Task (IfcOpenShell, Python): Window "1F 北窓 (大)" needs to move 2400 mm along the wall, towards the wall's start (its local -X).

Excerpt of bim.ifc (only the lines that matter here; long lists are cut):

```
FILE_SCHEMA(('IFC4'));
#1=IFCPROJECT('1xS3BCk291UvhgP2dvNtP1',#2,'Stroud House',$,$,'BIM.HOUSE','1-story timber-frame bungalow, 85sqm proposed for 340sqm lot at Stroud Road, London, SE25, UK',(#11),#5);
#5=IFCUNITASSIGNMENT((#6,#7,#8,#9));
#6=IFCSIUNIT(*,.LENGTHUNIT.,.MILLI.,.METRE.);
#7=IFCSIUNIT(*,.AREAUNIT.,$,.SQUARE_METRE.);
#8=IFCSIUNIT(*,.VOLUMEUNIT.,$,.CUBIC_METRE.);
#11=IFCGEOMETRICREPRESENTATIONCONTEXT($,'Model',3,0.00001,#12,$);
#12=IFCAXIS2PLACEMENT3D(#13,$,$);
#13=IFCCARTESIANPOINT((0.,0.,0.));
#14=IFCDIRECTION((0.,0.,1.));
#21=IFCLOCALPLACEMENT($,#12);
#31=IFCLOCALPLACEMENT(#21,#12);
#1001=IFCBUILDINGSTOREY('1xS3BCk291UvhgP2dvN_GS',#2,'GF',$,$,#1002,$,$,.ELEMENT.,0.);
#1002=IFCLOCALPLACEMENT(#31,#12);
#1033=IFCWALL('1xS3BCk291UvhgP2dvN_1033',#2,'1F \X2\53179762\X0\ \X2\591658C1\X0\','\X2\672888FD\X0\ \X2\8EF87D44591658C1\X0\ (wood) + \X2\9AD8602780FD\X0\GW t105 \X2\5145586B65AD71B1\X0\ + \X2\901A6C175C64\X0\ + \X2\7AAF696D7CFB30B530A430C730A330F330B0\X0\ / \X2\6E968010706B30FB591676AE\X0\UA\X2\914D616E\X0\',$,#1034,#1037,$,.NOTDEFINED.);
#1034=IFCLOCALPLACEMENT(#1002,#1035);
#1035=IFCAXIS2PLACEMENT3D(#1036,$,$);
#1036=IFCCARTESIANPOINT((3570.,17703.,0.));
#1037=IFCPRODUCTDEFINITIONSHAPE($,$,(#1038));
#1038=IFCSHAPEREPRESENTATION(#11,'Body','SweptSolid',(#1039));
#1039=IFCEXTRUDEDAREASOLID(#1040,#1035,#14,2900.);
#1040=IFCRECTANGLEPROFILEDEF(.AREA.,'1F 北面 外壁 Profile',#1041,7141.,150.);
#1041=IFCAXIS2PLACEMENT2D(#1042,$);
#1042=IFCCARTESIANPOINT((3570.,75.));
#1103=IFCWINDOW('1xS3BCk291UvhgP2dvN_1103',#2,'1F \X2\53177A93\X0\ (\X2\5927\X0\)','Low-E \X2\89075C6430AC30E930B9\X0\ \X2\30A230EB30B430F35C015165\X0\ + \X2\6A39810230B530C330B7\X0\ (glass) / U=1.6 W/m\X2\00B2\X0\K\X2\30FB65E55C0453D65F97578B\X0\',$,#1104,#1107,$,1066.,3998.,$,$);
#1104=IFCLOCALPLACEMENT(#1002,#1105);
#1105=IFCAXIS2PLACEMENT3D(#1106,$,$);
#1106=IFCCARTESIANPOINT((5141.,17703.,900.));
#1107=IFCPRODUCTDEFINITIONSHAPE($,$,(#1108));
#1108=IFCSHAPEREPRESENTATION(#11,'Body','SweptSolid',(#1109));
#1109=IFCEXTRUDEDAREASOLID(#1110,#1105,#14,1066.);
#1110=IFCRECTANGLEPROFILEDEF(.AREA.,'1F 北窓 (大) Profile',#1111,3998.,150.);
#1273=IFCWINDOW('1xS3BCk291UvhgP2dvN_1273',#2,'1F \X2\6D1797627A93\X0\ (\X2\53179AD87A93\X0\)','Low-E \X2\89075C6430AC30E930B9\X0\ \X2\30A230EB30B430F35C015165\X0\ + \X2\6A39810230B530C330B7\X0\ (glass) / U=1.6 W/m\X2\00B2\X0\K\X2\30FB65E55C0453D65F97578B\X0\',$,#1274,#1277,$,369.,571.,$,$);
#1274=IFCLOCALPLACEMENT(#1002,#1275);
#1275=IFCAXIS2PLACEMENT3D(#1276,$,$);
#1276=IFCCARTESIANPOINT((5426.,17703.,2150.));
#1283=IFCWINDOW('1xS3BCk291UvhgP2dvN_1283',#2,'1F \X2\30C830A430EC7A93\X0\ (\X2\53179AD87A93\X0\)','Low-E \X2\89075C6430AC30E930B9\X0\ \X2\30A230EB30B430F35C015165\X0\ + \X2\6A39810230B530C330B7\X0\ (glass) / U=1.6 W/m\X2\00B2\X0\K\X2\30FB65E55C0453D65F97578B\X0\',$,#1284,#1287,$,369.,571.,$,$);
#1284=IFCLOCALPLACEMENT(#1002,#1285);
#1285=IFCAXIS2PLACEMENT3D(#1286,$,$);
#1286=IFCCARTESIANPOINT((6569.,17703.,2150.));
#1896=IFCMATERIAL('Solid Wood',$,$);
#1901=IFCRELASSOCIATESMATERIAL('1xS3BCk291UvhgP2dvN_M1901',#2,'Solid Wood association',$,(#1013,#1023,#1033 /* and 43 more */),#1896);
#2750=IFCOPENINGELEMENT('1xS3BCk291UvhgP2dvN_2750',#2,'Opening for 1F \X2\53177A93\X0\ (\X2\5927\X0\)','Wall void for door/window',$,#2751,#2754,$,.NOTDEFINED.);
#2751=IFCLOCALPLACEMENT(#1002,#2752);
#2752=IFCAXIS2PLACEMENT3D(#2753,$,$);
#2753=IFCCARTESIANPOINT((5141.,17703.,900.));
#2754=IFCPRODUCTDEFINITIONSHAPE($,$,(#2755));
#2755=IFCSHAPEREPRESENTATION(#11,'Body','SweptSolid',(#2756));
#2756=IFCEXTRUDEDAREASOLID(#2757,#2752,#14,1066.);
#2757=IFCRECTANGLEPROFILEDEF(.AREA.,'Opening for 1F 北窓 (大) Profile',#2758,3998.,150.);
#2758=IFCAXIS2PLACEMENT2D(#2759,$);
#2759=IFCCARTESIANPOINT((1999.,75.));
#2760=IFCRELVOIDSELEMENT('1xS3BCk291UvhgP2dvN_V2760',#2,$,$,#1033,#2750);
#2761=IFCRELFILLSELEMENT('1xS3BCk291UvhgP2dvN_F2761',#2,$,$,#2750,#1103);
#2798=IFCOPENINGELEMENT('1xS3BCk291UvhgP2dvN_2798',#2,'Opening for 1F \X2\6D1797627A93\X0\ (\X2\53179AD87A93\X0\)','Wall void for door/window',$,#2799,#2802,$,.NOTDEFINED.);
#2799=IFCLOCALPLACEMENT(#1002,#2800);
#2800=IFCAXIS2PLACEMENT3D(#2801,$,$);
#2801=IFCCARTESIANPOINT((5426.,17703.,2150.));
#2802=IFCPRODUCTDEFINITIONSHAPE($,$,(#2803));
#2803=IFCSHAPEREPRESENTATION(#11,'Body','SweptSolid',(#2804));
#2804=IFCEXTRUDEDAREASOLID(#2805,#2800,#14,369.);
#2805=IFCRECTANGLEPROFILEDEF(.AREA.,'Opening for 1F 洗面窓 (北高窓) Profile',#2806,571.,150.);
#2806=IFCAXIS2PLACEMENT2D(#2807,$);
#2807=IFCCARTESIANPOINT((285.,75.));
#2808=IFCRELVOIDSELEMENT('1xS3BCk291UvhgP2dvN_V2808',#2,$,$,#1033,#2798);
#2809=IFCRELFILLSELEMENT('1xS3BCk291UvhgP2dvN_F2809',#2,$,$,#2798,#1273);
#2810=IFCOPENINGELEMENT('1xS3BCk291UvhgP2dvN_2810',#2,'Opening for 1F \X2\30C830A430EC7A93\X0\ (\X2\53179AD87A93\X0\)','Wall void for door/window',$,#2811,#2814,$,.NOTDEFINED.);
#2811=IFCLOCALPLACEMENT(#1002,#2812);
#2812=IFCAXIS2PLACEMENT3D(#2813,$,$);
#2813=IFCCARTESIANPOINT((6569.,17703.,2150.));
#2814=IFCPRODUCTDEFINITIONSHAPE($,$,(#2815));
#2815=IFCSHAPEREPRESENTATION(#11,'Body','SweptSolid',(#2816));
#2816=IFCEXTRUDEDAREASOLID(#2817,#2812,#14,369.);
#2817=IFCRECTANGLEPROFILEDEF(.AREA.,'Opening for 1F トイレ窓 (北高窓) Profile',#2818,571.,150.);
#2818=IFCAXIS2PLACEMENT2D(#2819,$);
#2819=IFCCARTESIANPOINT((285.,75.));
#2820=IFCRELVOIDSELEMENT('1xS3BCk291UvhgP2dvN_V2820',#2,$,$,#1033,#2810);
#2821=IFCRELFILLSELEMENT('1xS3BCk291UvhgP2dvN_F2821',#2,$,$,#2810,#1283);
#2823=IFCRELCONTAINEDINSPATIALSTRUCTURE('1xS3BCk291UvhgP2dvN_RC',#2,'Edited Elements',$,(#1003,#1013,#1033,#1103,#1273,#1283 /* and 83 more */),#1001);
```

```python
import ifcopenshell
import ifcopenshell.api.geometry
import ifcopenshell.util.placement
import ifcopenshell.util.unit

model = ifcopenshell.open("bim.ifc")
unit_scale = ifcopenshell.util.unit.calculate_unit_scale(model)

window = model.by_guid("1xS3BCk291UvhgP2dvN_1103")
opening = window.FillsVoids[0].RelatingOpeningElement
wall = opening.VoidsElements[0].RelatingBuildingElement

wall_matrix = ifcopenshell.util.placement.get_local_placement(wall.ObjectPlacement)
shift = wall_matrix[:3, 0] * -2.4 / unit_scale
before = ifcopenshell.util.placement.get_local_placement(window.ObjectPlacement)[:3, 3].copy()

# The window is not placed relative to its opening, so move both.
for product in (opening, window):
    matrix = ifcopenshell.util.placement.get_local_placement(product.ObjectPlacement)
    matrix[:3, 3] += shift
    ifcopenshell.api.geometry.edit_object_placement(model, product=product, matrix=matrix, is_si=False)

after = ifcopenshell.util.placement.get_local_placement(window.ObjectPlacement)[:3, 3]
print("window moved by", (after - before).round(3) + 0.0)

model.write("bim-out.ifc")
```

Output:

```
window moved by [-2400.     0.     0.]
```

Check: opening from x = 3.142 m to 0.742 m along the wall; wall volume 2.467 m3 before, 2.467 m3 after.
